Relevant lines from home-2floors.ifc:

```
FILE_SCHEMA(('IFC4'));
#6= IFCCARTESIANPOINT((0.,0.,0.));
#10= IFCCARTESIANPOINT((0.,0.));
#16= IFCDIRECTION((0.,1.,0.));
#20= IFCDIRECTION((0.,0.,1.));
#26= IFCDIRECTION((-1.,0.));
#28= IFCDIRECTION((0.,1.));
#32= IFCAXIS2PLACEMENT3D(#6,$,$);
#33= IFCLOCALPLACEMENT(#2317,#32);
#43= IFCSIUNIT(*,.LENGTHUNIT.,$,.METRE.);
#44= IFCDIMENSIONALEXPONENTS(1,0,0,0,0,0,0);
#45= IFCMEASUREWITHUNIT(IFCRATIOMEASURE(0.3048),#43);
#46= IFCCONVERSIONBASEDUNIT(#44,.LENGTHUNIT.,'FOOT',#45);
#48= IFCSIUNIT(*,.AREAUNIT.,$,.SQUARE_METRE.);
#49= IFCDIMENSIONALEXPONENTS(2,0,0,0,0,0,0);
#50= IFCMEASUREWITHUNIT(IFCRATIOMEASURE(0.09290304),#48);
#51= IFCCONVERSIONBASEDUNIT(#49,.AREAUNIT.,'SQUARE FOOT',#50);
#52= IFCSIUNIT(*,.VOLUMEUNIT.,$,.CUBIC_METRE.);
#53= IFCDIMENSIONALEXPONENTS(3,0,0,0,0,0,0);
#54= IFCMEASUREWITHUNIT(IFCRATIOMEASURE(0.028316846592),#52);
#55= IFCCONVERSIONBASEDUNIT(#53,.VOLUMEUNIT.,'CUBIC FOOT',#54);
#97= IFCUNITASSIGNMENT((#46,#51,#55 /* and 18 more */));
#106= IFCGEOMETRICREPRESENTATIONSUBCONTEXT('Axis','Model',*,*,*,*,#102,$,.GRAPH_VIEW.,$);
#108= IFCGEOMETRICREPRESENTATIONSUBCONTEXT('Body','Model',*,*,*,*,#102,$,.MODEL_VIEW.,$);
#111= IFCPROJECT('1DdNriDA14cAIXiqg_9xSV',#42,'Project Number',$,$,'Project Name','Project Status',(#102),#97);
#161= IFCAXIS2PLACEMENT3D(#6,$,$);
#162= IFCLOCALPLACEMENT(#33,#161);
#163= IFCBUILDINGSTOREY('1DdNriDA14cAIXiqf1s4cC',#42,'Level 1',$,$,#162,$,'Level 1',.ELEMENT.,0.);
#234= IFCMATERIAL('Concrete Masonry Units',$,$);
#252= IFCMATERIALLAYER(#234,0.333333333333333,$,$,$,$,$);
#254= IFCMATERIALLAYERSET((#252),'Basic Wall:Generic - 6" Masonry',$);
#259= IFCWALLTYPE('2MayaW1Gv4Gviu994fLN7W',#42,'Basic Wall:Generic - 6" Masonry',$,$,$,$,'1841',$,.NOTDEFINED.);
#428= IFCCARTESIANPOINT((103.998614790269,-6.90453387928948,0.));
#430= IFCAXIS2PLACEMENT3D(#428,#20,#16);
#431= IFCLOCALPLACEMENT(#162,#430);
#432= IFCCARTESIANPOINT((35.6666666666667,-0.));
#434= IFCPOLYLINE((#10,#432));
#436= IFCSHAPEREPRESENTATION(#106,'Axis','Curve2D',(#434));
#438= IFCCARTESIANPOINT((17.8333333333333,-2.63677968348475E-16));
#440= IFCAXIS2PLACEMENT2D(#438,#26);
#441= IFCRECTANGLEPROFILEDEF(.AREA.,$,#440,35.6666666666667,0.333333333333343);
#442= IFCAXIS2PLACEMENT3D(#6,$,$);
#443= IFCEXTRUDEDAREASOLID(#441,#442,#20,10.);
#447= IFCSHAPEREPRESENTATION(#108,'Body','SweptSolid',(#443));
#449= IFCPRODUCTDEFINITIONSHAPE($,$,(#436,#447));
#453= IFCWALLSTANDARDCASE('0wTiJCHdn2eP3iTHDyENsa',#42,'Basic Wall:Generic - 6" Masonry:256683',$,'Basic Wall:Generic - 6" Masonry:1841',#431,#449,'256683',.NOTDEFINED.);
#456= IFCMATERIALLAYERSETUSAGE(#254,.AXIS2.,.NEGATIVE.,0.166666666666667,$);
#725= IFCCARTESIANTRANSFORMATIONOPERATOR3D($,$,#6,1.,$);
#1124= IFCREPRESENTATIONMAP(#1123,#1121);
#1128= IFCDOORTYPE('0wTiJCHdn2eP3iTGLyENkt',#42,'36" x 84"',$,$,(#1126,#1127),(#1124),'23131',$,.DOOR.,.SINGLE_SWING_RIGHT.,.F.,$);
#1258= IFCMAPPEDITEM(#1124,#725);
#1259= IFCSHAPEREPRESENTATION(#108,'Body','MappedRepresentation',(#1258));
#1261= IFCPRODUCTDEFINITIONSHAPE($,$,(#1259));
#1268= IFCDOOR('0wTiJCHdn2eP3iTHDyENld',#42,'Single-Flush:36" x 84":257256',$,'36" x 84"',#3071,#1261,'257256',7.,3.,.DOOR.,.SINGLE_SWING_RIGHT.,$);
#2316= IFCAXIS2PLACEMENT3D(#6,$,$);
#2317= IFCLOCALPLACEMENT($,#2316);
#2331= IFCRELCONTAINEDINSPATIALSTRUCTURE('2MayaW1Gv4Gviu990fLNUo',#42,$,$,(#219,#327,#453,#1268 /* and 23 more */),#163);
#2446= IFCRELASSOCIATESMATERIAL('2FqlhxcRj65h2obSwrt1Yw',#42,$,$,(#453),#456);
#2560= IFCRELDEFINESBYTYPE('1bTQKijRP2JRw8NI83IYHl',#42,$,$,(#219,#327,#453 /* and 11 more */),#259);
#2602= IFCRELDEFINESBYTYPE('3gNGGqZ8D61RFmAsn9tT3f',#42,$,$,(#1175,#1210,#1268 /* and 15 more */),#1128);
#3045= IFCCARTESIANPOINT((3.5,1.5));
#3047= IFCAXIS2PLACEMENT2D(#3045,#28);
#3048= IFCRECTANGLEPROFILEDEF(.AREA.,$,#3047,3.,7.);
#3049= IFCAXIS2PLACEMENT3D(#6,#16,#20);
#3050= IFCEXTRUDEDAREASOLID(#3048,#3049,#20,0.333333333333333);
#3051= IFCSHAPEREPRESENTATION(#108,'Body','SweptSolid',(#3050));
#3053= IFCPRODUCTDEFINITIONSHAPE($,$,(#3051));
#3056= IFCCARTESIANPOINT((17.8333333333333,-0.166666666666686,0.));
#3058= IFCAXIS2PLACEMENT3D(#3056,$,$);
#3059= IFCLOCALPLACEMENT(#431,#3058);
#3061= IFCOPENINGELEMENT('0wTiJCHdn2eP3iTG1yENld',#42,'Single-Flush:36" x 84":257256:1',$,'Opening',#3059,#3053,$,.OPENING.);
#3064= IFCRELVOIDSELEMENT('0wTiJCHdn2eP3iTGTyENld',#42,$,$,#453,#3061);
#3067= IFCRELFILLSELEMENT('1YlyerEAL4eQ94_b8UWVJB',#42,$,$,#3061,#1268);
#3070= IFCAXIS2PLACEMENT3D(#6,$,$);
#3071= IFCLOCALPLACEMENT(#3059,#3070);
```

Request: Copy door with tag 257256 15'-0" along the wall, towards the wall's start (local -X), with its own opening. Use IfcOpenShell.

```python
import ifcopenshell
import ifcopenshell.api.feature
import ifcopenshell.api.geometry
import ifcopenshell.api.root
import ifcopenshell.geom
import ifcopenshell.util.element
import ifcopenshell.util.placement
import ifcopenshell.util.shape
import ifcopenshell.util.unit

model = ifcopenshell.open("home-2floors.ifc")
unit_scale = ifcopenshell.util.unit.calculate_unit_scale(model)
settings = ifcopenshell.geom.settings()


def volume(element):
    """Net volume in cubic metres, openings subtracted."""
    shape = ifcopenshell.geom.create_shape(settings, element)
    return ifcopenshell.util.shape.get_volume(shape.geometry)


def reuse_history(source, copy):
    """copy_class also copies each property set's owner history, people and application; keep the originals."""
    for rel in copy.IsDefinedBy:
        if rel.is_a("IfcRelDefinesByProperties") and (history := rel.RelatingPropertyDefinition.OwnerHistory):
            rel.RelatingPropertyDefinition.OwnerHistory = source.OwnerHistory
            ifcopenshell.util.element.remove_deep2(model, history)


door = model.by_guid("0wTiJCHdn2eP3iTHDyENld")
opening = door.FillsVoids[0].RelatingOpeningElement
wall = opening.VoidsElements[0].RelatingBuildingElement
before = volume(wall)
shift = ifcopenshell.util.placement.get_local_placement(wall.ObjectPlacement)[:3, 0] * -180 * 0.0254 / unit_scale

# copy_class copies the void relationship, type, container and properties, but no geometry.
new_opening = ifcopenshell.api.root.copy_class(model, product=opening)
new_opening.Representation = ifcopenshell.util.element.copy_deep(
    model, opening.Representation, exclude=["IfcGeometricRepresentationContext", "IfcRepresentationMap"]
)
new_opening.Name = 'Single-Flush:36" x 84"'
new_door = ifcopenshell.api.root.copy_class(model, product=door)
new_door.Representation = ifcopenshell.util.element.copy_deep(
    model, door.Representation, exclude=["IfcGeometricRepresentationContext", "IfcRepresentationMap"]
)
new_door.Name = 'Single-Flush:36" x 84"'
new_door.Tag = None
reuse_history(door, new_door)
ifcopenshell.api.feature.add_filling(model, opening=new_opening, element=new_door)

for old, new in ((opening, new_opening), (door, new_door)):
    matrix = ifcopenshell.util.placement.get_local_placement(old.ObjectPlacement)
    matrix[:3, 3] += shift
    ifcopenshell.api.geometry.edit_object_placement(model, product=new, matrix=matrix, is_si=False)

after = volume(wall)

print(f"wall volume {before:.3f} -> {after:.3f} m3")

model.write("home-2floors-out.ifc")
```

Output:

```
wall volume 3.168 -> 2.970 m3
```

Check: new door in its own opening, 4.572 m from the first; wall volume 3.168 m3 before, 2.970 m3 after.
